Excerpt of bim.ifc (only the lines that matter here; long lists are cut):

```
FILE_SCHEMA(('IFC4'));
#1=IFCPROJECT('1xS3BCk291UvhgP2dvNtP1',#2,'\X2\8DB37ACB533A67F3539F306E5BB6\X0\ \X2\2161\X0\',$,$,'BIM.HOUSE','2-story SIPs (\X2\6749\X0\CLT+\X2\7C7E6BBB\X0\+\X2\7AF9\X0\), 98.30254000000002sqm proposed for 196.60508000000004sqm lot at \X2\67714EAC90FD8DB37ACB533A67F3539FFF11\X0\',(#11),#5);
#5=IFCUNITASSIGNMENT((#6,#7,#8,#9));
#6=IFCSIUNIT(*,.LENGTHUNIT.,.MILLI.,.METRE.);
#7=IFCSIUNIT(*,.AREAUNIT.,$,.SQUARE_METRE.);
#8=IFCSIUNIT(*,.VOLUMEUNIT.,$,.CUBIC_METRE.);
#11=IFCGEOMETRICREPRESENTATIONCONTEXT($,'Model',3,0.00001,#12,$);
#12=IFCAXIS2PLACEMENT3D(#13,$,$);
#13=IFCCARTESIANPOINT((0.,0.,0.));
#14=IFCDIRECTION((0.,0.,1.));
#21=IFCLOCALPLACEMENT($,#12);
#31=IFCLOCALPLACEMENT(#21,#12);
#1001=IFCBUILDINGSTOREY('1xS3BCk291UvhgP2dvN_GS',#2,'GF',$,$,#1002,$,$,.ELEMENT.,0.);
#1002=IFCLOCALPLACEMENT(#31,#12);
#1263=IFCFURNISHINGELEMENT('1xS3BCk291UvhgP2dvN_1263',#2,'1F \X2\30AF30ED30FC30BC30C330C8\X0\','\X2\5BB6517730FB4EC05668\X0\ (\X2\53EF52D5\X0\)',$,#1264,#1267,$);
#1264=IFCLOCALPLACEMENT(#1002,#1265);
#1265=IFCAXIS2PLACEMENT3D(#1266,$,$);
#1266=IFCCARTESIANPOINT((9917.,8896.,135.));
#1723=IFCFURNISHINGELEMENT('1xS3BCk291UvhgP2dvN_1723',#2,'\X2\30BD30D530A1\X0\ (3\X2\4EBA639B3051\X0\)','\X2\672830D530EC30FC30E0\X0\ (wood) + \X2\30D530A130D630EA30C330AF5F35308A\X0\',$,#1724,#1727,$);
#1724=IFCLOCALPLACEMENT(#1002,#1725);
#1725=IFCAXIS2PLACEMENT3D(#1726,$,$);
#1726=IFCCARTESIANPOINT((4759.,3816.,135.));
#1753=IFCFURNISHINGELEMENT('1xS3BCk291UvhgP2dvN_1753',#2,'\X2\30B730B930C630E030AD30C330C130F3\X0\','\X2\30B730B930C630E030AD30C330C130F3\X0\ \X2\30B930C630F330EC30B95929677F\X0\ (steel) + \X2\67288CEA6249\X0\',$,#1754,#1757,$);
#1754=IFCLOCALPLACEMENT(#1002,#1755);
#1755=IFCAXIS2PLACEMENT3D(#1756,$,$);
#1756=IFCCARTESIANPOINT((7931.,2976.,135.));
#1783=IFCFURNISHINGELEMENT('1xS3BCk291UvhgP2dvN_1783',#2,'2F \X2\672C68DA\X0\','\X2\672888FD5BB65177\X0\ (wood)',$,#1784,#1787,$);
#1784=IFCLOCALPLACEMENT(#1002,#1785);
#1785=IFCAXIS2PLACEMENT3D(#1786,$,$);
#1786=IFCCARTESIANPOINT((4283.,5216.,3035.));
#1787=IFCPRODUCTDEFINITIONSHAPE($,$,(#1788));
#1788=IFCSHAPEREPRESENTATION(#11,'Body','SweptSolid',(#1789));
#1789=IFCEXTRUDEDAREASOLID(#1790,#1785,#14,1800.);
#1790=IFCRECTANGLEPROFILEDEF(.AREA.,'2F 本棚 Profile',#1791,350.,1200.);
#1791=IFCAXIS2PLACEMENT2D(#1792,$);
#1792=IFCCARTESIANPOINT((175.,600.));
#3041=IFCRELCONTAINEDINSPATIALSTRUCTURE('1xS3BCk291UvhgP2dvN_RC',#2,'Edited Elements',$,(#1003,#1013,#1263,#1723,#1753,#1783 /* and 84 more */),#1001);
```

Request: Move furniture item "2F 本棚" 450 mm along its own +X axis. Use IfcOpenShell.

```python
import ifcopenshell
import ifcopenshell.api.geometry
import ifcopenshell.util.placement
import ifcopenshell.util.unit

model = ifcopenshell.open("bim.ifc")
unit_scale = ifcopenshell.util.unit.calculate_unit_scale(model)

item = model.by_id(1783)
matrix = ifcopenshell.util.placement.get_local_placement(item.ObjectPlacement)
matrix[:3, 3] += matrix[:3, 0] * 0.45 / unit_scale
ifcopenshell.api.geometry.edit_object_placement(model, product=item, matrix=matrix, is_si=False)

print(ifcopenshell.util.placement.get_local_placement(item.ObjectPlacement).round(3) + 0.0)

model.write("bim_rev.ifc")
```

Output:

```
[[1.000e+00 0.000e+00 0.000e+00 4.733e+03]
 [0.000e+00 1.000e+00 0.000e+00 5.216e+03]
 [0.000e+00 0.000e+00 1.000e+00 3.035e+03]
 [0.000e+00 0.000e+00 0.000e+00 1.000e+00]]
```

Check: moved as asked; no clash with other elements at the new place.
